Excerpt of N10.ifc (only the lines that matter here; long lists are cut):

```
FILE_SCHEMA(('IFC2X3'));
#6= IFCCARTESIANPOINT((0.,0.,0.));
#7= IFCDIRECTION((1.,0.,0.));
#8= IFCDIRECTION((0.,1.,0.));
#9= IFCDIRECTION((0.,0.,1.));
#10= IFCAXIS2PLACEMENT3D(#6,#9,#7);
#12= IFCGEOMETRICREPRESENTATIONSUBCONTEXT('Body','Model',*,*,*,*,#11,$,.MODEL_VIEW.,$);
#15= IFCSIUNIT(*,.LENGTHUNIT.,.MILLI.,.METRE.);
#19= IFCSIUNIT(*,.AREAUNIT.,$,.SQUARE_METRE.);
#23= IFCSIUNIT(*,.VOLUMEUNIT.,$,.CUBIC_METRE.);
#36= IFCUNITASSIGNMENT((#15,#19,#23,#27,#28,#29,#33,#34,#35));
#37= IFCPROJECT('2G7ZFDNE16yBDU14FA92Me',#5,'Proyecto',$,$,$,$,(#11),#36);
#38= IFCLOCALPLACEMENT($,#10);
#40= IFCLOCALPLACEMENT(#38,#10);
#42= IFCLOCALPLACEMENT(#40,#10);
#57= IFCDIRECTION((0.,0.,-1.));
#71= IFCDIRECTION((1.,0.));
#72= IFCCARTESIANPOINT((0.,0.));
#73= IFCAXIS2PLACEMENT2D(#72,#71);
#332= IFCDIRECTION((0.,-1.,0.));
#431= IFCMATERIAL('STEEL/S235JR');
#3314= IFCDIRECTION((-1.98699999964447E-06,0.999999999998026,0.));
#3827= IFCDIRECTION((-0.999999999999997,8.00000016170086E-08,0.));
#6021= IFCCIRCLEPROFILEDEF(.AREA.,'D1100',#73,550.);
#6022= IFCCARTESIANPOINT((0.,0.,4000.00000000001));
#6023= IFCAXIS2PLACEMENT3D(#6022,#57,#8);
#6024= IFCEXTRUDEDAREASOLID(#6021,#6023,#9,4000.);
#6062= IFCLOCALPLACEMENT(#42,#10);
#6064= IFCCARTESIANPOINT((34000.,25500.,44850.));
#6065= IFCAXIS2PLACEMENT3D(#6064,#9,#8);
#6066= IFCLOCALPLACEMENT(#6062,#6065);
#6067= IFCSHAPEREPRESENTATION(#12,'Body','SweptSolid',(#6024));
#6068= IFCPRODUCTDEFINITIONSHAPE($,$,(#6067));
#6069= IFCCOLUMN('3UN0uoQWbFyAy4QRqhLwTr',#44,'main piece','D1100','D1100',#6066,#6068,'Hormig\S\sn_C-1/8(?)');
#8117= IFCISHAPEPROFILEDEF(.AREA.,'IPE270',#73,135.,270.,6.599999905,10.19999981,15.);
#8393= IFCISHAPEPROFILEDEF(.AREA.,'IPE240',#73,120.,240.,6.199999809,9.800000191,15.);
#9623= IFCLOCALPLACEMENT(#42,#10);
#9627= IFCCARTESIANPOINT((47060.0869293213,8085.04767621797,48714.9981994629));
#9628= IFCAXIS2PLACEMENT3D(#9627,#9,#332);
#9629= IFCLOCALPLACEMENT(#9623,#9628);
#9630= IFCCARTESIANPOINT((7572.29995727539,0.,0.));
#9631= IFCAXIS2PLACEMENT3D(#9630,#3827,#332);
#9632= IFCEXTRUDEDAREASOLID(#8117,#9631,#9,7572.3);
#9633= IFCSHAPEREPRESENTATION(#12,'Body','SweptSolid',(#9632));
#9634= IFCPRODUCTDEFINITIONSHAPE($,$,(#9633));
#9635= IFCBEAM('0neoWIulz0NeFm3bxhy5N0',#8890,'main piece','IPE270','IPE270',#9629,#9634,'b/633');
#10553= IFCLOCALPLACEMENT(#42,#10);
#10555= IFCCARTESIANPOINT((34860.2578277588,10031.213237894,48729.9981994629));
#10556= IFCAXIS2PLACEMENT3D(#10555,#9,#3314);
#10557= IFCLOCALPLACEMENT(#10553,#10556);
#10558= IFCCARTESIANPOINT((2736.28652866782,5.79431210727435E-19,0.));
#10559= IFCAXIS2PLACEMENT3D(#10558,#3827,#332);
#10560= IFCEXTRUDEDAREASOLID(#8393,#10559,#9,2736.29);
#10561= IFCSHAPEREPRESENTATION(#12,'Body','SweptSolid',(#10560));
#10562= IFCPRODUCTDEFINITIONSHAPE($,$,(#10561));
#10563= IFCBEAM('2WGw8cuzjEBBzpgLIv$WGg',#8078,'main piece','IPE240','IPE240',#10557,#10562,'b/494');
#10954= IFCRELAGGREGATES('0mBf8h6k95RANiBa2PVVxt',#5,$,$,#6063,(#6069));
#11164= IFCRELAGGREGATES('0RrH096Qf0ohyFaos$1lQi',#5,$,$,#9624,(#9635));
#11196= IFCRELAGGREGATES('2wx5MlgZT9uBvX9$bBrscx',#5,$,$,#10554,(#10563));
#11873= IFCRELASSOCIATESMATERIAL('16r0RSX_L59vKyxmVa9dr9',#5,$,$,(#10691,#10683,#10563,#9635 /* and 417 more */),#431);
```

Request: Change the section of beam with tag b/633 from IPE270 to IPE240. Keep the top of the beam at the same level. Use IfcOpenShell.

```python
import ifcopenshell
import ifcopenshell.util.element
import ifcopenshell.util.representation

model = ifcopenshell.open("N10.ifc")

member = model.by_guid("0neoWIulz0NeFm3bxhy5N0")
source = next(p for p in model.by_type("IfcIShapeProfileDef") if p.ProfileName == "IPE240")

body = ifcopenshell.util.representation.get_representation(member, "Model", "Body")
solid = body.Items[0]
old_profile = solid.SweptArea

# Copy the section's sizes but keep this member's own profile position.
profile = ifcopenshell.util.element.copy(model, source)
# Profiles are centred, so shift by half the change in depth to hold the top.
shift = (old_profile.OverallDepth - profile.OverallDepth) / 2
x, y = old_profile.Position.Location.Coordinates
up = (0.0, 1.0)  # upwards, in the solid's own plane
location = model.createIfcCartesianPoint((x + up[0] * shift, y + up[1] * shift))
profile.Position = model.createIfcAxis2Placement2D(location, old_profile.Position.RefDirection)
solid.SweptArea = profile
if not model.get_total_inverses(old_profile):
    ifcopenshell.util.element.remove_deep2(model, old_profile)
member.Description = member.Description.replace("IPE270", "IPE240")
member.ObjectType = member.ObjectType.replace("IPE270", "IPE240")

print(solid.SweptArea)

model.write("N10-out.ifc")
```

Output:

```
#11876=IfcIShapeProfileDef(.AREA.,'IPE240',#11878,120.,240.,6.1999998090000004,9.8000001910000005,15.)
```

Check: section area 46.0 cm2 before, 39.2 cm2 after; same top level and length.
